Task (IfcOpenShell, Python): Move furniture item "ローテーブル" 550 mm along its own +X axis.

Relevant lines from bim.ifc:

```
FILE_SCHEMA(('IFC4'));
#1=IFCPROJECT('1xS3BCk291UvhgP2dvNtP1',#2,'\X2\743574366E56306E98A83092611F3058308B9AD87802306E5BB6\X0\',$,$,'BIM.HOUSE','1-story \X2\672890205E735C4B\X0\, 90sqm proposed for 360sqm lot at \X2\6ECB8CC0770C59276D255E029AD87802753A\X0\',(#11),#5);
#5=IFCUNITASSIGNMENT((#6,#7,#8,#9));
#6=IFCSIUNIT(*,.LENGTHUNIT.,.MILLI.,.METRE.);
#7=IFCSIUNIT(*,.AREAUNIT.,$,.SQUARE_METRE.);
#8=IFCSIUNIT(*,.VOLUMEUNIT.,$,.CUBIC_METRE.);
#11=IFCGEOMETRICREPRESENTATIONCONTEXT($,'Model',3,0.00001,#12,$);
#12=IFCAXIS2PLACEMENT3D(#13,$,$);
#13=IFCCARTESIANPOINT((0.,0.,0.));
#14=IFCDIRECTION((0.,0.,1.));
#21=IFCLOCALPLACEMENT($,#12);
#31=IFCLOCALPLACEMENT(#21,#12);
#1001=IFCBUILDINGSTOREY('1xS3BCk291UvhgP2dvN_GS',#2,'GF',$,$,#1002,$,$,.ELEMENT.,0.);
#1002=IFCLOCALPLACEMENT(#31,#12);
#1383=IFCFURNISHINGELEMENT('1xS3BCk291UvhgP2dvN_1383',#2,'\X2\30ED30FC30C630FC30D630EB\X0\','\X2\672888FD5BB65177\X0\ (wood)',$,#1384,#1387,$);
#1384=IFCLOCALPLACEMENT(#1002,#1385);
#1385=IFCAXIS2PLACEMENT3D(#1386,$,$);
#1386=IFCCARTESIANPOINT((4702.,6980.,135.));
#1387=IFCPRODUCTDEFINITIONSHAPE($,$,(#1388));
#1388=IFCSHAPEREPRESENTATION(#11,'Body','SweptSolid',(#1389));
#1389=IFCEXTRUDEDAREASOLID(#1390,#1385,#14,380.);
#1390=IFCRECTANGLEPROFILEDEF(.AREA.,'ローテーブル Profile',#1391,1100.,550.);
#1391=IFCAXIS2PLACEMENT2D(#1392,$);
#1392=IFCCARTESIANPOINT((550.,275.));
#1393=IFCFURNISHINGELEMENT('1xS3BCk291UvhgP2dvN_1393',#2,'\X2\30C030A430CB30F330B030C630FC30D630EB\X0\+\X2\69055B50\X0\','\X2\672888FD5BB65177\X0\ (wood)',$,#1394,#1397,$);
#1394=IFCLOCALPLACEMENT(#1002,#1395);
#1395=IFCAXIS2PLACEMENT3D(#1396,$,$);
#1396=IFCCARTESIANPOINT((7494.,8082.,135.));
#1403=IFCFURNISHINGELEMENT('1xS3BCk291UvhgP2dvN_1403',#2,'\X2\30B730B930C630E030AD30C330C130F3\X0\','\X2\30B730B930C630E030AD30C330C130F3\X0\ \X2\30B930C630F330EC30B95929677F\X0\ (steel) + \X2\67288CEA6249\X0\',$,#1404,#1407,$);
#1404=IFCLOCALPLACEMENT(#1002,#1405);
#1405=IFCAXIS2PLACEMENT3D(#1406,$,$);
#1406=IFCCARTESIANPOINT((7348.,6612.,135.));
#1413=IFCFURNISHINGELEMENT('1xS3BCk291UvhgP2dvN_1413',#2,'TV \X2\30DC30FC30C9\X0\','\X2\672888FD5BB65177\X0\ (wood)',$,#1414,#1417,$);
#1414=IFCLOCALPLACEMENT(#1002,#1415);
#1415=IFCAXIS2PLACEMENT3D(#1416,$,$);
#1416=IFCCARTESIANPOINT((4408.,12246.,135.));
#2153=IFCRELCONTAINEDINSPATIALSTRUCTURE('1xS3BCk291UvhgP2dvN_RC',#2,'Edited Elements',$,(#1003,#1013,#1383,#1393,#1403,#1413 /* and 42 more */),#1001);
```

```python
import ifcopenshell
import ifcopenshell.api.geometry
import ifcopenshell.util.placement
import ifcopenshell.util.unit

model = ifcopenshell.open("bim.ifc")
unit_scale = ifcopenshell.util.unit.calculate_unit_scale(model)

item = model.by_id(1383)
matrix = ifcopenshell.util.placement.get_local_placement(item.ObjectPlacement)
matrix[:3, 3] += matrix[:3, 0] * 0.55 / unit_scale
ifcopenshell.api.geometry.edit_object_placement(model, product=item, matrix=matrix, is_si=False)

print(ifcopenshell.util.placement.get_local_placement(item.ObjectPlacement).round(3) + 0.0)

model.write("bim-out.ifc")
```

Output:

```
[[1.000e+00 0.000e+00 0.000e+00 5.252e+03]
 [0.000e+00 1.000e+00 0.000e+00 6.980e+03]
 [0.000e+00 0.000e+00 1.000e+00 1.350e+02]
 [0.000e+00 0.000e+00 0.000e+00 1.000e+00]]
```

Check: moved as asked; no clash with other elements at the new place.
